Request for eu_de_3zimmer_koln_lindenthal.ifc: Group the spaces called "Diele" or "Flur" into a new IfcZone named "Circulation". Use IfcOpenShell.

First a look at what the model holds.

```python
import ifcopenshell

model = ifcopenshell.open("eu_de_3zimmer_koln_lindenthal.ifc")
print(model.schema)
seen = {}
for space in model.by_type("IfcSpace"):
    seen[space.LongName] = seen.get(space.LongName, 0) + 1
for name, count in sorted(seen.items(), key=str):
    print(count, "x", name)
print("zones:", [z.Name for z in model.by_type("IfcZone")][:20])
```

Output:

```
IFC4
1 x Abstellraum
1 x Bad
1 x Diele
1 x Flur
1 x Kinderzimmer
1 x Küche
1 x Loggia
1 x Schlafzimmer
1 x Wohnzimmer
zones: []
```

```python
import ifcopenshell
import ifcopenshell.api.group
import ifcopenshell.api.root

model = ifcopenshell.open("eu_de_3zimmer_koln_lindenthal.ifc")

names = {"Diele", "Flur"}
spaces = [s for s in model.by_type("IfcSpace") if s.LongName in names]

zone = ifcopenshell.api.root.create_entity(model, ifc_class="IfcZone", name="Circulation")
ifcopenshell.api.group.assign_group(model, products=spaces, group=zone)
print(len(spaces), "spaces in", zone.Name)

model.write("eu_de_3zimmer_koln_lindenthal-out.ifc")
```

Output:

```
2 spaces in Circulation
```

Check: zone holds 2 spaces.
